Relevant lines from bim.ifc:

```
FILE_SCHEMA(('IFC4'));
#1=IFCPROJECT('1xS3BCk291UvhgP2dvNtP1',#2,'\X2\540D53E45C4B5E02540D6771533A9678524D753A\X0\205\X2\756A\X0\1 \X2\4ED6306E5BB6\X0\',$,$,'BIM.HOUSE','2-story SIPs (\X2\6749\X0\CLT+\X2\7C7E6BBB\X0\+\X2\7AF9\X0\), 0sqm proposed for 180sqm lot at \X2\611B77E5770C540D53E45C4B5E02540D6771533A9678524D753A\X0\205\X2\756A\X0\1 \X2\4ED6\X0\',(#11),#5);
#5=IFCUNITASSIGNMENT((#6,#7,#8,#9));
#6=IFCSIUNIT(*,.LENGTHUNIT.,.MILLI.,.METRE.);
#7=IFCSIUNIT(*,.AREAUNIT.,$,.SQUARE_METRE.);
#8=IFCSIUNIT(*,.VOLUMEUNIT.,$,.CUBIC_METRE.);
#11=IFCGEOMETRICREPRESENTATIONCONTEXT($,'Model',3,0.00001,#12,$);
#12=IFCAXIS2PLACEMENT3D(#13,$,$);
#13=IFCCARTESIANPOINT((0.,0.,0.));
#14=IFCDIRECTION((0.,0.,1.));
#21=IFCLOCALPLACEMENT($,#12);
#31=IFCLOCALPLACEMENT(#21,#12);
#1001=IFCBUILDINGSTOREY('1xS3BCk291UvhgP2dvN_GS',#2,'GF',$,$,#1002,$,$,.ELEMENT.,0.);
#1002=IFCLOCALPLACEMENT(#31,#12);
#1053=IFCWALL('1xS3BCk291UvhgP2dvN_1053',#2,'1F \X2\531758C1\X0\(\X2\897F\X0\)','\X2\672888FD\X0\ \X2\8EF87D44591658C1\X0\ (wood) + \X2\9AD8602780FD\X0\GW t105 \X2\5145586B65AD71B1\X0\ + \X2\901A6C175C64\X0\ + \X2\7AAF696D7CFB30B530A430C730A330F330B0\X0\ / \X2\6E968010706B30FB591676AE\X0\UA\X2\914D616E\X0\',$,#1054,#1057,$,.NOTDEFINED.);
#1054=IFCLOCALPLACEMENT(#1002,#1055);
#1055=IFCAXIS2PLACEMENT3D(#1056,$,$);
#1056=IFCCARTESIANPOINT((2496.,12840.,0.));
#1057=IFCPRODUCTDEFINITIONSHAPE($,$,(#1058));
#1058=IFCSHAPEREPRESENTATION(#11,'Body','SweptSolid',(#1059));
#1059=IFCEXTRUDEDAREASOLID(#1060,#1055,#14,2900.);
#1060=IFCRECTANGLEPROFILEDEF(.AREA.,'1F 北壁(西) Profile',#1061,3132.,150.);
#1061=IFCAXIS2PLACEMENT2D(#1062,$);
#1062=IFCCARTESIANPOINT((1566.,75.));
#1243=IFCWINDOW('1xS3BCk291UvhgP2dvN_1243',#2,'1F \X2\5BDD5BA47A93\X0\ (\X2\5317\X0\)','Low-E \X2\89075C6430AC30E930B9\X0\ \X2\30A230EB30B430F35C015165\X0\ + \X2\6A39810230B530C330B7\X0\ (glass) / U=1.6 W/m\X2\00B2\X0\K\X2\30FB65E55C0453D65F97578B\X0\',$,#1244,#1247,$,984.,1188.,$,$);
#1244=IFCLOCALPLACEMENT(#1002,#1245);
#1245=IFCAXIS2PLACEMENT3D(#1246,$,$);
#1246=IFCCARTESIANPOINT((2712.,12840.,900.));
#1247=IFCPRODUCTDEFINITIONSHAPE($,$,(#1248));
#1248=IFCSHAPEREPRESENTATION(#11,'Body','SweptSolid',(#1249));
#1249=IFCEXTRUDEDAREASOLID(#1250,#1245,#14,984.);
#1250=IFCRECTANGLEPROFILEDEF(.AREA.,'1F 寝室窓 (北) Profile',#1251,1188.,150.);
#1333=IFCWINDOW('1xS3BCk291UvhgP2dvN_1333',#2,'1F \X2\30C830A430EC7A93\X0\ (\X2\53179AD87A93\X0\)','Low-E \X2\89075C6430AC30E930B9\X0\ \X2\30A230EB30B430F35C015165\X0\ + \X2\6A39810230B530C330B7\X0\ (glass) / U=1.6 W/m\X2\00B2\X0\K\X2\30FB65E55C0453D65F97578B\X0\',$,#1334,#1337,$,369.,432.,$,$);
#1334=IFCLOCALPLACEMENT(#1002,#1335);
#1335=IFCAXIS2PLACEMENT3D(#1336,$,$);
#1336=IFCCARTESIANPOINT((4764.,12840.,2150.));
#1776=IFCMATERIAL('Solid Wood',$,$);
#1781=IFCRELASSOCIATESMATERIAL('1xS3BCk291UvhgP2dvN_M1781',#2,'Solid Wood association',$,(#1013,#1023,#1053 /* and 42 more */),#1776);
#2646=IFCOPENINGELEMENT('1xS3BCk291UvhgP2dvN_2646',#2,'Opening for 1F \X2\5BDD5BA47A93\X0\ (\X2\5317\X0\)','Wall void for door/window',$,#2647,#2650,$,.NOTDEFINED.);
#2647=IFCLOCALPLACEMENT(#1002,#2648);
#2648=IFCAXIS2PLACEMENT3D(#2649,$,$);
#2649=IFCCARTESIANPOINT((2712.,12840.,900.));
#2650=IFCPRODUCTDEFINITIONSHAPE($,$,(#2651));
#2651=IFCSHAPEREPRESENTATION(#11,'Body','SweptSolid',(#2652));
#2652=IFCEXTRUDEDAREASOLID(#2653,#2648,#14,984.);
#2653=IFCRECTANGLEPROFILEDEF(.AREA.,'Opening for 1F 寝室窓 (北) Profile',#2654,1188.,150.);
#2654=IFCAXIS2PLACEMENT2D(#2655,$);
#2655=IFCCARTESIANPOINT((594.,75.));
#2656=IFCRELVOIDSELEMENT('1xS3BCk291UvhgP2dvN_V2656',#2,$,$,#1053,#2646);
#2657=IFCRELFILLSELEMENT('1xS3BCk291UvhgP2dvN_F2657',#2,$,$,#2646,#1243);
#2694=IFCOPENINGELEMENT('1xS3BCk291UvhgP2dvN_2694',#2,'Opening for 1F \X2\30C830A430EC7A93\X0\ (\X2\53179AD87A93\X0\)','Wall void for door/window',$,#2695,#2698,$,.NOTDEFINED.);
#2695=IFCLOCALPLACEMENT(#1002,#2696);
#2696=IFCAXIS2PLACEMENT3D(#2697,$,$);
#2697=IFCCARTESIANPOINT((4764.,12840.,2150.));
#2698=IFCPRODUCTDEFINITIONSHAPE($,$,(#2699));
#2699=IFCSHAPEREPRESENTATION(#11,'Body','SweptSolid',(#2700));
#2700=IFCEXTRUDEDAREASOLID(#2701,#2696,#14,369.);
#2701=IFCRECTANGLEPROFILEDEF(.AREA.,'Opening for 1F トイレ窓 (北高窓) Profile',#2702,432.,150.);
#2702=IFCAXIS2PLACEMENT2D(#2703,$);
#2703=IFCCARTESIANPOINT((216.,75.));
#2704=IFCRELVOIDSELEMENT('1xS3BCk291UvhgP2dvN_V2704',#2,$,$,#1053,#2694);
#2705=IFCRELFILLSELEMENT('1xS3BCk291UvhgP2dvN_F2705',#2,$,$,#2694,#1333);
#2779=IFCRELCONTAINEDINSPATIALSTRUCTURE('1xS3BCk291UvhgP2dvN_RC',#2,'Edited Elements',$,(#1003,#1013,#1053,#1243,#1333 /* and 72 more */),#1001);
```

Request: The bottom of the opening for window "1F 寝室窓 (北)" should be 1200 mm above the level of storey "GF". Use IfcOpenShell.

```python
import numpy as np
import ifcopenshell
import ifcopenshell.api.geometry
import ifcopenshell.geom
import ifcopenshell.util.element
import ifcopenshell.util.placement
import ifcopenshell.util.shape
import ifcopenshell.util.unit

model = ifcopenshell.open("bim.ifc")
unit_scale = ifcopenshell.util.unit.calculate_unit_scale(model)

window = model.by_guid("1xS3BCk291UvhgP2dvN_1243")
opening = window.FillsVoids[0].RelatingOpeningElement
storey = ifcopenshell.util.element.get_container(window, ifc_class="IfcBuildingStorey")
level = ifcopenshell.util.placement.get_local_placement(storey.ObjectPlacement)[2, 3]

# The opening's origin need not be at the sill, so measure its lowest point.
shape = ifcopenshell.geom.create_shape(ifcopenshell.geom.settings(), opening)
bottom = ifcopenshell.util.shape.get_shape_bottom_elevation(shape, shape.geometry) / unit_scale
dz = level + 1200.0 - bottom

shift = np.array([0.0, 0.0, dz])
# The window is not placed relative to its opening, so move both.
for product in (opening, window):
    matrix = ifcopenshell.util.placement.get_local_placement(product.ObjectPlacement)
    matrix[:3, 3] += shift
    ifcopenshell.api.geometry.edit_object_placement(model, product=product, matrix=matrix, is_si=False)

print(f"moved by {dz * unit_scale:+.3f} m")

model.write("bim-out.ifc")
```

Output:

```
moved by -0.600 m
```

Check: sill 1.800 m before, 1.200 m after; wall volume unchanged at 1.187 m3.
